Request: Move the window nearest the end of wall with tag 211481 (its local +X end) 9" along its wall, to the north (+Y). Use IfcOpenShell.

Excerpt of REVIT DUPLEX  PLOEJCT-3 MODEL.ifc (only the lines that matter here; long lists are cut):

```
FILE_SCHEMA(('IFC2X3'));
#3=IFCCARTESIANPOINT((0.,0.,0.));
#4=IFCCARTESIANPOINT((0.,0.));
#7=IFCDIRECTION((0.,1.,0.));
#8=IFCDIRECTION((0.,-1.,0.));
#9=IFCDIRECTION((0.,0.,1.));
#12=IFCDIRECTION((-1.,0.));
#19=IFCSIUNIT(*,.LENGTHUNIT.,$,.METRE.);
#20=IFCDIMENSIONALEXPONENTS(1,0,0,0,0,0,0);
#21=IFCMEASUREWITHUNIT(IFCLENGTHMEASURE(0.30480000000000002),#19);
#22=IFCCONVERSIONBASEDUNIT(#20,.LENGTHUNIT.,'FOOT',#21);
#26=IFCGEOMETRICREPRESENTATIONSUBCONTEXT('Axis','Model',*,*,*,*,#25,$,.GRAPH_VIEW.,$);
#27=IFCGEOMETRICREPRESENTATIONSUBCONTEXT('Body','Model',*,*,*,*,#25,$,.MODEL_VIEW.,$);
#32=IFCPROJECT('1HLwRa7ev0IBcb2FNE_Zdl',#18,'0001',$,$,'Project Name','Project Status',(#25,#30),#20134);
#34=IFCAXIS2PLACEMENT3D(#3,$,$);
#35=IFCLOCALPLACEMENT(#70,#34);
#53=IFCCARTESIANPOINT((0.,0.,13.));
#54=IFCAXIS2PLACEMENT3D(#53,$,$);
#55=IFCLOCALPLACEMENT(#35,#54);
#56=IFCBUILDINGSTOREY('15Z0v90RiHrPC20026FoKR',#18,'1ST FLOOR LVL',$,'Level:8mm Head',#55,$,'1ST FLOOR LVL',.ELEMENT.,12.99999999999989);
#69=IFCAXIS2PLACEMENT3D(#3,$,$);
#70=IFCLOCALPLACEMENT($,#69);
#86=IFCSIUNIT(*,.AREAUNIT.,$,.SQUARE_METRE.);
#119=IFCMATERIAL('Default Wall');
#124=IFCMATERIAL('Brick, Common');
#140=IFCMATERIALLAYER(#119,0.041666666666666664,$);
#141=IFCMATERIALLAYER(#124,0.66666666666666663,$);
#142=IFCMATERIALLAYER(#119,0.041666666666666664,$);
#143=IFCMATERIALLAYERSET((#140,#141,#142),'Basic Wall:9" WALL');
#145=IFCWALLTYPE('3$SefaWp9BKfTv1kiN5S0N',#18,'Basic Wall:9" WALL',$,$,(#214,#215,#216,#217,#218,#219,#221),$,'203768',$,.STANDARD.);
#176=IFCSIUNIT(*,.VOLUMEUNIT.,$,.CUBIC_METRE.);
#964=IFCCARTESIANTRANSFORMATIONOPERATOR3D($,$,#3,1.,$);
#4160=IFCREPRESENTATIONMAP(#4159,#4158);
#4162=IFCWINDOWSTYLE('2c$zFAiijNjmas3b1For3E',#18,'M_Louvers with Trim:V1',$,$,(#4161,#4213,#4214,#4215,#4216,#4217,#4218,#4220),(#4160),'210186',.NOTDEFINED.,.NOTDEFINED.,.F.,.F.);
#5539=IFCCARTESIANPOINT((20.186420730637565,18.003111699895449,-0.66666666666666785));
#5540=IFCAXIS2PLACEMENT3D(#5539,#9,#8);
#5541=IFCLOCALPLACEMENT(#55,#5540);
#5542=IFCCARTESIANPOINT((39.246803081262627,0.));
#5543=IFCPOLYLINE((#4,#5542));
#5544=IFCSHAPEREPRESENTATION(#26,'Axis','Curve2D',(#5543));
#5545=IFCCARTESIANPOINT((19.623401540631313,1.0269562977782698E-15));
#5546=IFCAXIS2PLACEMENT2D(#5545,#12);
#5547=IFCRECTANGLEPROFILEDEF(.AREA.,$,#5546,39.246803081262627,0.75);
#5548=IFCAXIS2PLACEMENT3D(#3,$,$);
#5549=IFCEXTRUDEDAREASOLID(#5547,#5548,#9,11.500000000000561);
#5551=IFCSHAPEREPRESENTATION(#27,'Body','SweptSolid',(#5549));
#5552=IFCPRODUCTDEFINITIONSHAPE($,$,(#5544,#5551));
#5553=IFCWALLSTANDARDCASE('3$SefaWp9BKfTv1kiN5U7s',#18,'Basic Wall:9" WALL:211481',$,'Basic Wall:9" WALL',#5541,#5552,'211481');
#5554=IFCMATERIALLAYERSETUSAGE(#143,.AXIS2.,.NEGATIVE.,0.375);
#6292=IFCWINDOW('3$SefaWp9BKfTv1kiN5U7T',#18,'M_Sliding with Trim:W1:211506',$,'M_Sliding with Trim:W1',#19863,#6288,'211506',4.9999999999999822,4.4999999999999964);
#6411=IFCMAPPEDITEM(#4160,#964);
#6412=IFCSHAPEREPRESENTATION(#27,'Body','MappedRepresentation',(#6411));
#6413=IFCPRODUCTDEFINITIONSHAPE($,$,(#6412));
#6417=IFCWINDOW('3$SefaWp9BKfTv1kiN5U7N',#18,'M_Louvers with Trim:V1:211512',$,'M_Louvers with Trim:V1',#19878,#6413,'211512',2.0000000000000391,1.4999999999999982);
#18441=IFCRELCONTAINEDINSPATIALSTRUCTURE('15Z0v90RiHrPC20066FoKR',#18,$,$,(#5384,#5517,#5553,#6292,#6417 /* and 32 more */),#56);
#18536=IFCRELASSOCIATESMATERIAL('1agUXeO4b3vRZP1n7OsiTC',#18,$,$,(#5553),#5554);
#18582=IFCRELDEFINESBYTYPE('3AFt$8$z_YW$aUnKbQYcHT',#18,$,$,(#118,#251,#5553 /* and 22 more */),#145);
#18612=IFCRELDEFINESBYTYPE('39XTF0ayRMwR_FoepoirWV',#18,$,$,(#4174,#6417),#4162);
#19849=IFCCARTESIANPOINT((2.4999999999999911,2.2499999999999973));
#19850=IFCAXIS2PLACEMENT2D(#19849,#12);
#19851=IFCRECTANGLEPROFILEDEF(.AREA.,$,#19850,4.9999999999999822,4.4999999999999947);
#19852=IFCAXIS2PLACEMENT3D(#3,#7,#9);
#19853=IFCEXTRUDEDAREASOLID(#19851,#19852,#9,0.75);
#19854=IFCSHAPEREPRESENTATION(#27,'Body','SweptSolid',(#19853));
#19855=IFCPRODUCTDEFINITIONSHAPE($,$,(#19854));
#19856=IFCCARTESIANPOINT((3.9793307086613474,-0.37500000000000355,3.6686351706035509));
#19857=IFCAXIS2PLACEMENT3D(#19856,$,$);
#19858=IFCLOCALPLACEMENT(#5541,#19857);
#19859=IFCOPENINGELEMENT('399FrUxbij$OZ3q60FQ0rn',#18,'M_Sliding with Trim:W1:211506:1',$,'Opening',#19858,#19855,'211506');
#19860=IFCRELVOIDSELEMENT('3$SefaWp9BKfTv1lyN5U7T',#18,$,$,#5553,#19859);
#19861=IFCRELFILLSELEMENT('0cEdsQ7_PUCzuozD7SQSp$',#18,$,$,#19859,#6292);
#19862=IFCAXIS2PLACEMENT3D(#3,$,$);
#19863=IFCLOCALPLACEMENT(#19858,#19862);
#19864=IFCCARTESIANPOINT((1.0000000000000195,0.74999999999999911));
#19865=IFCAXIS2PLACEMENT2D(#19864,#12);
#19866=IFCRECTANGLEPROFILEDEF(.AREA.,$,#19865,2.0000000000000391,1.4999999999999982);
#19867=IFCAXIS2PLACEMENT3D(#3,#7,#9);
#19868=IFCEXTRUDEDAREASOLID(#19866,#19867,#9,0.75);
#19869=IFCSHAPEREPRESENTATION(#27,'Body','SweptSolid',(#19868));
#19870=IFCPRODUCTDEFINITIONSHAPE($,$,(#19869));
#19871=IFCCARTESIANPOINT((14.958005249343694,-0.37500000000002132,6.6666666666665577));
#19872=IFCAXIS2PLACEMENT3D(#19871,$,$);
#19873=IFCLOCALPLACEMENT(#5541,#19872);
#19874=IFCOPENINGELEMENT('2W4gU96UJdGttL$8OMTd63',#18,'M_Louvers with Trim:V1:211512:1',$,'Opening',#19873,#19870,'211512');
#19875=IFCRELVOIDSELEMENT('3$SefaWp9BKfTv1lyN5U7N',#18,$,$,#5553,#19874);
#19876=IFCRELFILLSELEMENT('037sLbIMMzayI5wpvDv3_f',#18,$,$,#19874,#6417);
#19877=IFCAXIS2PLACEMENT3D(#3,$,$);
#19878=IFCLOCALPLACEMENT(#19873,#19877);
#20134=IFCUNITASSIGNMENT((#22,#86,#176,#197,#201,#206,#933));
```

```python
import ifcopenshell
import ifcopenshell.api.geometry
import ifcopenshell.util.placement
import ifcopenshell.util.unit

model = ifcopenshell.open("REVIT DUPLEX  PLOEJCT-3 MODEL.ifc")
unit_scale = ifcopenshell.util.unit.calculate_unit_scale(model)

window = model.by_id(6417)
opening = window.FillsVoids[0].RelatingOpeningElement
wall = opening.VoidsElements[0].RelatingBuildingElement

wall_matrix = ifcopenshell.util.placement.get_local_placement(wall.ObjectPlacement)
shift = wall_matrix[:3, 0] * -9 * 0.0254 / unit_scale
before = ifcopenshell.util.placement.get_local_placement(window.ObjectPlacement)[:3, 3].copy()

# The window is placed relative to its opening, so it follows when the opening moves.
matrix = ifcopenshell.util.placement.get_local_placement(opening.ObjectPlacement)
matrix[:3, 3] += shift
ifcopenshell.api.geometry.edit_object_placement(
    model, product=opening, matrix=matrix, is_si=False, should_transform_children=True
)

after = ifcopenshell.util.placement.get_local_placement(window.ObjectPlacement)[:3, 3]
print("window moved by", (after - before).round(3) + 0.0)

model.write("REVIT DUPLEX  PLOEJCT-3 MODEL-out.ifc")
```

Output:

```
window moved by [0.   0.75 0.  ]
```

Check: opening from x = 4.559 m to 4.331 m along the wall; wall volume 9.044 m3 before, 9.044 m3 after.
